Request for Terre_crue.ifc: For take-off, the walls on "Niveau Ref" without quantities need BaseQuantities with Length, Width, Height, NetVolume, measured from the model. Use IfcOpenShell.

First a look at what the model holds.

```python
import ifcopenshell
import ifcopenshell.util.element
import ifcopenshell.util.unit

model = ifcopenshell.open("Terre_crue.ifc")
print(model.schema)
for unit_type in ("LENGTHUNIT", "AREAUNIT", "VOLUMEUNIT"):
    print(unit_type, ifcopenshell.util.unit.calculate_unit_scale(model, unit_type))
storey = next(s for s in model.by_type("IfcBuildingStorey") if s.Name == "Niveau Ref")
walls = [e for e in ifcopenshell.util.element.get_decomposition(storey) if e.is_a("IfcWall")]
for e in sorted(walls, key=lambda e: e.id()):
    print(e.id(), e.is_a(), e.Name, list(ifcopenshell.util.element.get_psets(e, qtos_only=True)), sep=" | ")
```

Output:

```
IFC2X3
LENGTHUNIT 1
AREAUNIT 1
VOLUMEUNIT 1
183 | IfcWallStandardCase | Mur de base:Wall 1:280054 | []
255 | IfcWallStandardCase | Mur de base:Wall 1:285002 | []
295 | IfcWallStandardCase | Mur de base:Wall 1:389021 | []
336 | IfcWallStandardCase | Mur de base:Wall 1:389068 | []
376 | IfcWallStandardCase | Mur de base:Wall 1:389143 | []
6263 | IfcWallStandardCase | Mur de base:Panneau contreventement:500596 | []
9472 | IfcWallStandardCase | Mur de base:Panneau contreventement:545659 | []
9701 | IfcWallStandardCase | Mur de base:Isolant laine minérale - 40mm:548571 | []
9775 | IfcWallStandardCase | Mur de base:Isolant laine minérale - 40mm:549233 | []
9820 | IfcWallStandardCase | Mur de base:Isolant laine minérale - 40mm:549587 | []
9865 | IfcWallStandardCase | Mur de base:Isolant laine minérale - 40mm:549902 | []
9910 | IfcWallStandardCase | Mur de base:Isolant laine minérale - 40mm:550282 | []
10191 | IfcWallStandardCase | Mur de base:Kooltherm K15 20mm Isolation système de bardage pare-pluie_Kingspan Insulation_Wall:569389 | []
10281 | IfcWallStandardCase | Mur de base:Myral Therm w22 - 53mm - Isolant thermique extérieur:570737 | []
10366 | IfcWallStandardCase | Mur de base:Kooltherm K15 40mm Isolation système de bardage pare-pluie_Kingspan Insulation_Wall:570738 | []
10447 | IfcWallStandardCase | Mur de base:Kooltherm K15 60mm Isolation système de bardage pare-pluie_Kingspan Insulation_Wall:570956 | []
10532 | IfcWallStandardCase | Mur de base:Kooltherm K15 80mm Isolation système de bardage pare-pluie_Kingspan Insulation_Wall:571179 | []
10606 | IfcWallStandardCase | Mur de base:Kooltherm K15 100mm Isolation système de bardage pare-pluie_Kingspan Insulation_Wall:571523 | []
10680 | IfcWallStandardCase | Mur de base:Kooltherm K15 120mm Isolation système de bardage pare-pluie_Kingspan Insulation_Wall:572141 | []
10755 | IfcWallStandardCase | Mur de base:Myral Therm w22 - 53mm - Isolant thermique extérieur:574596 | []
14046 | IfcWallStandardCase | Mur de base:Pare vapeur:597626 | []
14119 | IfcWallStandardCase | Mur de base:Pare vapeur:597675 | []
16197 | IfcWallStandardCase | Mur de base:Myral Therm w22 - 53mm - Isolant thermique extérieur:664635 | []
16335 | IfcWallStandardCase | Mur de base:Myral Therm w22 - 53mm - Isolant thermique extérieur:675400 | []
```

```python
import ifcopenshell
import ifcopenshell.api.pset
import ifcopenshell.geom
import ifcopenshell.util.element
import ifcopenshell.util.shape
import ifcopenshell.util.unit

model = ifcopenshell.open("Terre_crue.ifc")
unit_scale = ifcopenshell.util.unit.calculate_unit_scale(model)
volume_scale = ifcopenshell.util.unit.calculate_unit_scale(model, "VOLUMEUNIT")
settings = ifcopenshell.geom.settings()

storey = next(s for s in model.by_type("IfcBuildingStorey") if s.Name == "Niveau Ref")
walls = [e for e in ifcopenshell.util.element.get_decomposition(storey) if e.is_a("IfcWall")]

for e in sorted(walls, key=lambda e: e.id()):
    if ifcopenshell.util.element.get_psets(e, qtos_only=True, should_inherit=False):
        continue
    # Geometry comes back in metres, in the element's own axes.
    shape = ifcopenshell.geom.create_shape(settings, e)
    values = {
        "Length": ifcopenshell.util.shape.get_x(shape.geometry) / unit_scale,
        "Width": ifcopenshell.util.shape.get_y(shape.geometry) / unit_scale,
        "Height": ifcopenshell.util.shape.get_z(shape.geometry) / unit_scale,
        "NetVolume": ifcopenshell.util.shape.get_volume(shape.geometry) / volume_scale,
    }
    qto = ifcopenshell.api.pset.add_qto(model, product=e, name="BaseQuantities")
    ifcopenshell.api.pset.edit_qto(model, qto=qto, properties=values)
    print(e.id(), {k: round(v, 3) for k, v in values.items()})

model.write("Terre_crue_v2.ifc")
```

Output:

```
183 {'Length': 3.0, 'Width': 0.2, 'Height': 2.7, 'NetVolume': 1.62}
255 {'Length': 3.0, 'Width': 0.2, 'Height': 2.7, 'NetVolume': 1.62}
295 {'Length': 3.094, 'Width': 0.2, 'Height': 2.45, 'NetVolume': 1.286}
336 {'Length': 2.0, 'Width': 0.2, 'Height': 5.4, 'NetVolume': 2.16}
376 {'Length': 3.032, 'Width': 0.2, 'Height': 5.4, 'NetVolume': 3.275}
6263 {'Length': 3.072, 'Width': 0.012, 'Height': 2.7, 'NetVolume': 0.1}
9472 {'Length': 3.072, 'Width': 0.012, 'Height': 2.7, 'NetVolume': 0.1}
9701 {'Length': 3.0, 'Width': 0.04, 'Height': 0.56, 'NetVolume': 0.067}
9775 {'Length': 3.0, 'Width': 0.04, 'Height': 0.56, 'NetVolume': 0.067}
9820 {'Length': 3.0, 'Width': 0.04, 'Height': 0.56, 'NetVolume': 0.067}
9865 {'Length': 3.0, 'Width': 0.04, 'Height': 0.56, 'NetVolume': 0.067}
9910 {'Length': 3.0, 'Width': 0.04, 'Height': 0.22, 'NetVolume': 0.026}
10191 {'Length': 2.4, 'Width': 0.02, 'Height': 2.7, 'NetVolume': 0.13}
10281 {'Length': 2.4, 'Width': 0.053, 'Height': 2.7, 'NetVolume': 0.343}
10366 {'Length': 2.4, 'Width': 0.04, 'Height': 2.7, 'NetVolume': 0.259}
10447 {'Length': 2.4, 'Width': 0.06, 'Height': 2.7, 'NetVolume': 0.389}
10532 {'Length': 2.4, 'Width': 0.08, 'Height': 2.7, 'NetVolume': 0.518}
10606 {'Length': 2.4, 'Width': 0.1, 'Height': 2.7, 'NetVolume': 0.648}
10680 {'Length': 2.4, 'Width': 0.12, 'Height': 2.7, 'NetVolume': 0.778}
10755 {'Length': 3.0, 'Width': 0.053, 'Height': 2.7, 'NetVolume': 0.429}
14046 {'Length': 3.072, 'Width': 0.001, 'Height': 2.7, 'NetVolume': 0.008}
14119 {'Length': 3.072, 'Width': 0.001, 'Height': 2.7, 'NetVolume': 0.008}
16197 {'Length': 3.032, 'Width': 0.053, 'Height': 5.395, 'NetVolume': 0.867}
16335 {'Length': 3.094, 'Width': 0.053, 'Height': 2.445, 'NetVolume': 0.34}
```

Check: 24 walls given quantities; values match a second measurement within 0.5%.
